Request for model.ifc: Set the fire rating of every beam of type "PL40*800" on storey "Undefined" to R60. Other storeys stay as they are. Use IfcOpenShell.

First a look at what the model holds.

```python
import ifcopenshell
import ifcopenshell.util.element

model = ifcopenshell.open("model.ifc")
print(model.schema)
storey = next(s for s in model.by_type("IfcBuildingStorey") if s.Name == "Undefined")
beams = [e for e in ifcopenshell.util.element.get_decomposition(storey) if e.is_a("IfcBeam")]
seen = {}
for e in beams:
    element_type = ifcopenshell.util.element.get_type(e)
    key = (element_type.Name if element_type != e and element_type else None, ifcopenshell.util.element.get_pset(e, "Pset_BeamCommon", "FireRating"))
    seen[key] = seen.get(key, 0) + 1
for (name, value), count in sorted(seen.items(), key=str):
    print(count, "x", name, "|", value)
```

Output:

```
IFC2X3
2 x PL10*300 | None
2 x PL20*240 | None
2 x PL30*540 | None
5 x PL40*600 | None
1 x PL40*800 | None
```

```python
import ifcopenshell
import ifcopenshell.api.pset
import ifcopenshell.util.element

model = ifcopenshell.open("model.ifc")

storey = next(s for s in model.by_type("IfcBuildingStorey") if s.Name == "Undefined")
beams = [e for e in ifcopenshell.util.element.get_decomposition(storey) if e.is_a("IfcBeam")]

count = 0
for e in beams:
    element_type = ifcopenshell.util.element.get_type(e)
    if element_type in (None, e) or element_type.Name != "PL40*800":
        continue
    # add_pset returns the element's existing set when there is one.
    pset = ifcopenshell.api.pset.add_pset(model, product=e, name="Pset_BeamCommon")
    ifcopenshell.api.pset.edit_pset(model, pset=pset, properties={"FireRating": "R60"})
    count += 1

print(count, "beams updated")

model.write("model_updated.ifc")
```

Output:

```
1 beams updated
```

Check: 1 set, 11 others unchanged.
